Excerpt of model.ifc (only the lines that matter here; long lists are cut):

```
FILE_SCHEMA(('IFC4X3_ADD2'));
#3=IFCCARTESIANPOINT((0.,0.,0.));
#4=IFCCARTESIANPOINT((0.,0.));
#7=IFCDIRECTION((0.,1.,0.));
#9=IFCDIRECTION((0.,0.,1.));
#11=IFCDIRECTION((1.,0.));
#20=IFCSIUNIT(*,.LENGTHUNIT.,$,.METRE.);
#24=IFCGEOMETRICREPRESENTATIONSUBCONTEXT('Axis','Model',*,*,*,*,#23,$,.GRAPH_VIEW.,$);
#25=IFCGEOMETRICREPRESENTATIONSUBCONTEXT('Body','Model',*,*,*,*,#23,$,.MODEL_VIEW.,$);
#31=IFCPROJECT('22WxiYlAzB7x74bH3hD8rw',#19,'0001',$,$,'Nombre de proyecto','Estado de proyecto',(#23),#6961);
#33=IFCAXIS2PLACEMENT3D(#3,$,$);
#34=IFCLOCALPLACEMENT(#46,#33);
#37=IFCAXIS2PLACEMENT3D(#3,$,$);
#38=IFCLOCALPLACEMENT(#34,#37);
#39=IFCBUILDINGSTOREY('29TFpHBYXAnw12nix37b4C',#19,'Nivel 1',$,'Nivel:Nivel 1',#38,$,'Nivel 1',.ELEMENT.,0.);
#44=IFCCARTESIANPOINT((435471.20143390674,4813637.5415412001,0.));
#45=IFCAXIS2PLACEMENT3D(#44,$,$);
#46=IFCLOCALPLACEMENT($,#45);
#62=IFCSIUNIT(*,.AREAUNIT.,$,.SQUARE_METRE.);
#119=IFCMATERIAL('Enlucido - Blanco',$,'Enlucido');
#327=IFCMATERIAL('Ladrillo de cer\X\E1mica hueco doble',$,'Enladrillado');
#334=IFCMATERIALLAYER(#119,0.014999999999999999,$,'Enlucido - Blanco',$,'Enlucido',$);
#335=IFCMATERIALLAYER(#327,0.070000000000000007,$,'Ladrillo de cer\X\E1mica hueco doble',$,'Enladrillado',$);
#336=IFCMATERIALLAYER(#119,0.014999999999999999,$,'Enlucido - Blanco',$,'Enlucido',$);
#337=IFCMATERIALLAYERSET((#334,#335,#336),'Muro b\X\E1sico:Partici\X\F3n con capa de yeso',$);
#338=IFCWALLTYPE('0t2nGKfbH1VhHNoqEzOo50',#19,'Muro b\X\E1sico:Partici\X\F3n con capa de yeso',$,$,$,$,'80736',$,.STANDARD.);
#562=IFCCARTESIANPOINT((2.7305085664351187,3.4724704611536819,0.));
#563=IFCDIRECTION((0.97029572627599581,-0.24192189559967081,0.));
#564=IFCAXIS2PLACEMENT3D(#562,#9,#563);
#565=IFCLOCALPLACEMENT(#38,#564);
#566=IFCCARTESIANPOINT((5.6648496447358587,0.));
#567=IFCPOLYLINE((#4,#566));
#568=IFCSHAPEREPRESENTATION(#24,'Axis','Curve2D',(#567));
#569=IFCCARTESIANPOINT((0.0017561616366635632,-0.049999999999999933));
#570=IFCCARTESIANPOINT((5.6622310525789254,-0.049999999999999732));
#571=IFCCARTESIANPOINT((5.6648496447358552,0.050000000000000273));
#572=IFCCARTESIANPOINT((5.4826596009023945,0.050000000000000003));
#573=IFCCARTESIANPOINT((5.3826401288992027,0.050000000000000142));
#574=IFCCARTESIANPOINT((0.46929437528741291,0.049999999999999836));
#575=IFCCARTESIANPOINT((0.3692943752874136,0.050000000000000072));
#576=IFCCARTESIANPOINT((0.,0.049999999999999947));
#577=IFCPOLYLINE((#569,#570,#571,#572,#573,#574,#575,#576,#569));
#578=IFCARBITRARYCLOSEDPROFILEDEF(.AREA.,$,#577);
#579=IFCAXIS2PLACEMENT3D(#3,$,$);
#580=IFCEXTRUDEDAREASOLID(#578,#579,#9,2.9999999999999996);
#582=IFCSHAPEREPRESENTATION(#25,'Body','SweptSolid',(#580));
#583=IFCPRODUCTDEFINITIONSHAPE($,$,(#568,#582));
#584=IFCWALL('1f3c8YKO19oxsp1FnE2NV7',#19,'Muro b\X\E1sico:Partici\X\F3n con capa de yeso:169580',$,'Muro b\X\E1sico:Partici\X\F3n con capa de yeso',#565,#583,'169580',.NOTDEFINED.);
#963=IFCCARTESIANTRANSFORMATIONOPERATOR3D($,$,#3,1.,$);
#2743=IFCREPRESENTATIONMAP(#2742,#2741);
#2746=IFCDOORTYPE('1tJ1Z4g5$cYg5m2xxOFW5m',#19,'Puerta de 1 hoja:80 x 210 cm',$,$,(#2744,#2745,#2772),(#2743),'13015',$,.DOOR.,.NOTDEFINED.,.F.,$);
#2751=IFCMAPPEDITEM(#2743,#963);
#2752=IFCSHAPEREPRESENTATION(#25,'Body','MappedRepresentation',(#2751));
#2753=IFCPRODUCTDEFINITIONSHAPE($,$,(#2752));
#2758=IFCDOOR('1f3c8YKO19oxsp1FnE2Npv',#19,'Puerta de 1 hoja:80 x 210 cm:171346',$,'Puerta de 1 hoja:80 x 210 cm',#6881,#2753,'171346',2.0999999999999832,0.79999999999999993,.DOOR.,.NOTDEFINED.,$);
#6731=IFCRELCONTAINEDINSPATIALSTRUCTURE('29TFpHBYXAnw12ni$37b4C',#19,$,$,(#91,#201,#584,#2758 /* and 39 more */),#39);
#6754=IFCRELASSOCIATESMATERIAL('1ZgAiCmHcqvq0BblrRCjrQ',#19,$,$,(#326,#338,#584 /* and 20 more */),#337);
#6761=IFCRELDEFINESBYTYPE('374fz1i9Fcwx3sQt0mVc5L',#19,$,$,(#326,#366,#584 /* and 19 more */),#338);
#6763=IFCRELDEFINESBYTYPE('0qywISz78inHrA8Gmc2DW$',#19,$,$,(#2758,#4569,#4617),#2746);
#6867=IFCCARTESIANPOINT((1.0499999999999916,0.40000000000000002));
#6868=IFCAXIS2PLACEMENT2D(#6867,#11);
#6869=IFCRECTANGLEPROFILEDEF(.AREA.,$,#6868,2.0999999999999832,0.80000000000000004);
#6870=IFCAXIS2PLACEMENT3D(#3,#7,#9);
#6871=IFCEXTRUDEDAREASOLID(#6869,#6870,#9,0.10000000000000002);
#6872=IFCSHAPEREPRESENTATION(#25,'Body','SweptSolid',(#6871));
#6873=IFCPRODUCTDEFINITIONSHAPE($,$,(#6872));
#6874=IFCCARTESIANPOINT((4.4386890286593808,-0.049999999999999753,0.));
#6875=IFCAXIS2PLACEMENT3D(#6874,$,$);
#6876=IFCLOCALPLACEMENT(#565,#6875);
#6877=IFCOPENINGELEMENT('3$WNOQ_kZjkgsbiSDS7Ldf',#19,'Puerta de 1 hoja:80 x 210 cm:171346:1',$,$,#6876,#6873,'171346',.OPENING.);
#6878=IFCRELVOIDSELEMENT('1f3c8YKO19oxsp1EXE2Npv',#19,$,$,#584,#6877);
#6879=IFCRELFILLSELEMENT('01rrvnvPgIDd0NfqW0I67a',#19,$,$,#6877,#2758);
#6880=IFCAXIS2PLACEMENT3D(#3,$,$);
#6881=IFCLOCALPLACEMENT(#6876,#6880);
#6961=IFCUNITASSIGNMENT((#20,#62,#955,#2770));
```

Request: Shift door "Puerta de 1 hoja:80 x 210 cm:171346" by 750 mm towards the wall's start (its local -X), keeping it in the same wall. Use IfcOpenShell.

```python
import ifcopenshell
import ifcopenshell.api.geometry
import ifcopenshell.util.placement
import ifcopenshell.util.unit

model = ifcopenshell.open("model.ifc")
unit_scale = ifcopenshell.util.unit.calculate_unit_scale(model)

door = model.by_guid("1f3c8YKO19oxsp1FnE2Npv")
opening = door.FillsVoids[0].RelatingOpeningElement
wall = opening.VoidsElements[0].RelatingBuildingElement

wall_matrix = ifcopenshell.util.placement.get_local_placement(wall.ObjectPlacement)
shift = wall_matrix[:3, 0] * -0.75 / unit_scale
before = ifcopenshell.util.placement.get_local_placement(door.ObjectPlacement)[:3, 3].copy()

# The door is placed relative to its opening, so it follows when the opening moves.
matrix = ifcopenshell.util.placement.get_local_placement(opening.ObjectPlacement)
matrix[:3, 3] += shift
ifcopenshell.api.geometry.edit_object_placement(
    model, product=opening, matrix=matrix, is_si=False, should_transform_children=True
)

after = ifcopenshell.util.placement.get_local_placement(door.ObjectPlacement)[:3, 3]
print("door moved by", (after - before).round(3) + 0.0)

model.write("model-out.ifc")
```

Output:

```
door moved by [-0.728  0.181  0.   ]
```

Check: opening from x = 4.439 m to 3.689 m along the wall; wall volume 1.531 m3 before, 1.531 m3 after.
